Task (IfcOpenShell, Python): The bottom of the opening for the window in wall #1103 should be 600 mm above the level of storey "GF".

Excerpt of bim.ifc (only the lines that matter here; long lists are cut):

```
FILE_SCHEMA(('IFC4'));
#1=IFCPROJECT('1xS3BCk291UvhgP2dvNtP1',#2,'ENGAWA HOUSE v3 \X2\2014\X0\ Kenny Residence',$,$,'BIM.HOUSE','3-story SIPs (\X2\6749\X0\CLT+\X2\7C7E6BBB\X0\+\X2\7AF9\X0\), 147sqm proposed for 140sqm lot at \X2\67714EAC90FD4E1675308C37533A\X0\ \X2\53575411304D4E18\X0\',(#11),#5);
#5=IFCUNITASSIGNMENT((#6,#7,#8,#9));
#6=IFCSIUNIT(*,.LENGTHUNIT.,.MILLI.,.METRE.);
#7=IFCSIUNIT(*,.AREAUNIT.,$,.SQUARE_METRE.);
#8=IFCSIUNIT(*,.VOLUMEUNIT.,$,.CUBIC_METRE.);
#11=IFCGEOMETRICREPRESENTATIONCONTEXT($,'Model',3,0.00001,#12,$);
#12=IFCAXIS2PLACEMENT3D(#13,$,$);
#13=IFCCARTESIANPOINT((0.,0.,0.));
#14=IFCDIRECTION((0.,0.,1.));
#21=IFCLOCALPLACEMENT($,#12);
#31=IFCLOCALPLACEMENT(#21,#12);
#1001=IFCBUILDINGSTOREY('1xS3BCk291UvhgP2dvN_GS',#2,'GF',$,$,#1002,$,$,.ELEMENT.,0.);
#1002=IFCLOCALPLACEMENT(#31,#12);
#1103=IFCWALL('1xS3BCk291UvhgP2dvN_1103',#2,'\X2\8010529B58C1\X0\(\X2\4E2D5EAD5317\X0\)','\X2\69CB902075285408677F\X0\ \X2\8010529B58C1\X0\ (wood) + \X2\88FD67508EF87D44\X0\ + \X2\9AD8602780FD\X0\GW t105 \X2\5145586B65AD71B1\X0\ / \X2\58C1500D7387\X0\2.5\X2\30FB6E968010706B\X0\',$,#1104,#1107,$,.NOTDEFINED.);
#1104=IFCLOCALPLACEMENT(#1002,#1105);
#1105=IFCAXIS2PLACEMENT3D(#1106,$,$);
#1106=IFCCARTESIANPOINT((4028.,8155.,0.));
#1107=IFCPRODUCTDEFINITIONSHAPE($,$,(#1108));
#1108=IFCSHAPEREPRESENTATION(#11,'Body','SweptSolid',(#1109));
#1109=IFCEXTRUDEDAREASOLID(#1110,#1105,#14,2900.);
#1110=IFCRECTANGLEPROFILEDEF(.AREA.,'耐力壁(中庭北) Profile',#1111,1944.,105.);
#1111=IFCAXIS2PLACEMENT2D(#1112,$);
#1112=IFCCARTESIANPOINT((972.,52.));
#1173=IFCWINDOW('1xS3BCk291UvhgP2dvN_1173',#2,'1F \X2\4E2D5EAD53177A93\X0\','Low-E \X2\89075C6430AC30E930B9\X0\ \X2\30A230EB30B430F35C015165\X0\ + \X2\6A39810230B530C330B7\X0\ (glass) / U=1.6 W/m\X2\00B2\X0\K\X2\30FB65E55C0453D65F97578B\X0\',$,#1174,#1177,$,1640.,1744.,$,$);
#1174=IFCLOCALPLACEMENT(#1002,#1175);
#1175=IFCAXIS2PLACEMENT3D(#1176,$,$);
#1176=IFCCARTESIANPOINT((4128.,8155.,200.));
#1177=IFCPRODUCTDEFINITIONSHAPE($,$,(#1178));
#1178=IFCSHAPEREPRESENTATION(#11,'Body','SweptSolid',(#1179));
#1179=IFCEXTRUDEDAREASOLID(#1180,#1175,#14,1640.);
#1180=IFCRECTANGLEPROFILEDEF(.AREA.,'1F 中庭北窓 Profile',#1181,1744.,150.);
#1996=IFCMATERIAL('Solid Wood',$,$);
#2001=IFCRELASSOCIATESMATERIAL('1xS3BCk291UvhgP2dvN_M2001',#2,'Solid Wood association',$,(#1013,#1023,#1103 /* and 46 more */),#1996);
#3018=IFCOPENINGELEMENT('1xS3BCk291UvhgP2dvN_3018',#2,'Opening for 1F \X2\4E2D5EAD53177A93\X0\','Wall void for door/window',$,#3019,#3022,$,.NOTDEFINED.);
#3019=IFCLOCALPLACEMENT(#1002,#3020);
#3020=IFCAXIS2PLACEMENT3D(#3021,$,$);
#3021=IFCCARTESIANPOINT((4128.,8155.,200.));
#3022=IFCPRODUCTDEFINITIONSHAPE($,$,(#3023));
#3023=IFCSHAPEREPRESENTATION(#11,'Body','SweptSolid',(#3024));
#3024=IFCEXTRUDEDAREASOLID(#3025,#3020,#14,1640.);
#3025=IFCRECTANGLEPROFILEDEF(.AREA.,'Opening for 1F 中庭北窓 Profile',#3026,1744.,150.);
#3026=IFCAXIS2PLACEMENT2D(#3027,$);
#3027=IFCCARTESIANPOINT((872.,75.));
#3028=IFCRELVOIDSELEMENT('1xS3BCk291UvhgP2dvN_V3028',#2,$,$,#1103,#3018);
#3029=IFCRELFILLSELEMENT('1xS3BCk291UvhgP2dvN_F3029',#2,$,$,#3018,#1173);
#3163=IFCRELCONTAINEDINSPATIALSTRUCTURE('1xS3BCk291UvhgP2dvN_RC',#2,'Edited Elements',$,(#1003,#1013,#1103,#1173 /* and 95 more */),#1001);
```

```python
import numpy as np
import ifcopenshell
import ifcopenshell.api.geometry
import ifcopenshell.geom
import ifcopenshell.util.element
import ifcopenshell.util.placement
import ifcopenshell.util.shape
import ifcopenshell.util.unit

model = ifcopenshell.open("bim.ifc")
unit_scale = ifcopenshell.util.unit.calculate_unit_scale(model)

window = model.by_guid("1xS3BCk291UvhgP2dvN_1173")
opening = window.FillsVoids[0].RelatingOpeningElement
storey = ifcopenshell.util.element.get_container(window, ifc_class="IfcBuildingStorey")
level = ifcopenshell.util.placement.get_local_placement(storey.ObjectPlacement)[2, 3]

# The opening's origin need not be at the sill, so measure its lowest point.
shape = ifcopenshell.geom.create_shape(ifcopenshell.geom.settings(), opening)
bottom = ifcopenshell.util.shape.get_shape_bottom_elevation(shape, shape.geometry) / unit_scale
dz = level + 0.6 / unit_scale - bottom

shift = np.array([0.0, 0.0, dz])
# The window is not placed relative to its opening, so move both.
for product in (opening, window):
    matrix = ifcopenshell.util.placement.get_local_placement(product.ObjectPlacement)
    matrix[:3, 3] += shift
    ifcopenshell.api.geometry.edit_object_placement(model, product=product, matrix=matrix, is_si=False)

print(f"moved by {dz * unit_scale:+.3f} m")

model.write("bim_updated.ifc")
```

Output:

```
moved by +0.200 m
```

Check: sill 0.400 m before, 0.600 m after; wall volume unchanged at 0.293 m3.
